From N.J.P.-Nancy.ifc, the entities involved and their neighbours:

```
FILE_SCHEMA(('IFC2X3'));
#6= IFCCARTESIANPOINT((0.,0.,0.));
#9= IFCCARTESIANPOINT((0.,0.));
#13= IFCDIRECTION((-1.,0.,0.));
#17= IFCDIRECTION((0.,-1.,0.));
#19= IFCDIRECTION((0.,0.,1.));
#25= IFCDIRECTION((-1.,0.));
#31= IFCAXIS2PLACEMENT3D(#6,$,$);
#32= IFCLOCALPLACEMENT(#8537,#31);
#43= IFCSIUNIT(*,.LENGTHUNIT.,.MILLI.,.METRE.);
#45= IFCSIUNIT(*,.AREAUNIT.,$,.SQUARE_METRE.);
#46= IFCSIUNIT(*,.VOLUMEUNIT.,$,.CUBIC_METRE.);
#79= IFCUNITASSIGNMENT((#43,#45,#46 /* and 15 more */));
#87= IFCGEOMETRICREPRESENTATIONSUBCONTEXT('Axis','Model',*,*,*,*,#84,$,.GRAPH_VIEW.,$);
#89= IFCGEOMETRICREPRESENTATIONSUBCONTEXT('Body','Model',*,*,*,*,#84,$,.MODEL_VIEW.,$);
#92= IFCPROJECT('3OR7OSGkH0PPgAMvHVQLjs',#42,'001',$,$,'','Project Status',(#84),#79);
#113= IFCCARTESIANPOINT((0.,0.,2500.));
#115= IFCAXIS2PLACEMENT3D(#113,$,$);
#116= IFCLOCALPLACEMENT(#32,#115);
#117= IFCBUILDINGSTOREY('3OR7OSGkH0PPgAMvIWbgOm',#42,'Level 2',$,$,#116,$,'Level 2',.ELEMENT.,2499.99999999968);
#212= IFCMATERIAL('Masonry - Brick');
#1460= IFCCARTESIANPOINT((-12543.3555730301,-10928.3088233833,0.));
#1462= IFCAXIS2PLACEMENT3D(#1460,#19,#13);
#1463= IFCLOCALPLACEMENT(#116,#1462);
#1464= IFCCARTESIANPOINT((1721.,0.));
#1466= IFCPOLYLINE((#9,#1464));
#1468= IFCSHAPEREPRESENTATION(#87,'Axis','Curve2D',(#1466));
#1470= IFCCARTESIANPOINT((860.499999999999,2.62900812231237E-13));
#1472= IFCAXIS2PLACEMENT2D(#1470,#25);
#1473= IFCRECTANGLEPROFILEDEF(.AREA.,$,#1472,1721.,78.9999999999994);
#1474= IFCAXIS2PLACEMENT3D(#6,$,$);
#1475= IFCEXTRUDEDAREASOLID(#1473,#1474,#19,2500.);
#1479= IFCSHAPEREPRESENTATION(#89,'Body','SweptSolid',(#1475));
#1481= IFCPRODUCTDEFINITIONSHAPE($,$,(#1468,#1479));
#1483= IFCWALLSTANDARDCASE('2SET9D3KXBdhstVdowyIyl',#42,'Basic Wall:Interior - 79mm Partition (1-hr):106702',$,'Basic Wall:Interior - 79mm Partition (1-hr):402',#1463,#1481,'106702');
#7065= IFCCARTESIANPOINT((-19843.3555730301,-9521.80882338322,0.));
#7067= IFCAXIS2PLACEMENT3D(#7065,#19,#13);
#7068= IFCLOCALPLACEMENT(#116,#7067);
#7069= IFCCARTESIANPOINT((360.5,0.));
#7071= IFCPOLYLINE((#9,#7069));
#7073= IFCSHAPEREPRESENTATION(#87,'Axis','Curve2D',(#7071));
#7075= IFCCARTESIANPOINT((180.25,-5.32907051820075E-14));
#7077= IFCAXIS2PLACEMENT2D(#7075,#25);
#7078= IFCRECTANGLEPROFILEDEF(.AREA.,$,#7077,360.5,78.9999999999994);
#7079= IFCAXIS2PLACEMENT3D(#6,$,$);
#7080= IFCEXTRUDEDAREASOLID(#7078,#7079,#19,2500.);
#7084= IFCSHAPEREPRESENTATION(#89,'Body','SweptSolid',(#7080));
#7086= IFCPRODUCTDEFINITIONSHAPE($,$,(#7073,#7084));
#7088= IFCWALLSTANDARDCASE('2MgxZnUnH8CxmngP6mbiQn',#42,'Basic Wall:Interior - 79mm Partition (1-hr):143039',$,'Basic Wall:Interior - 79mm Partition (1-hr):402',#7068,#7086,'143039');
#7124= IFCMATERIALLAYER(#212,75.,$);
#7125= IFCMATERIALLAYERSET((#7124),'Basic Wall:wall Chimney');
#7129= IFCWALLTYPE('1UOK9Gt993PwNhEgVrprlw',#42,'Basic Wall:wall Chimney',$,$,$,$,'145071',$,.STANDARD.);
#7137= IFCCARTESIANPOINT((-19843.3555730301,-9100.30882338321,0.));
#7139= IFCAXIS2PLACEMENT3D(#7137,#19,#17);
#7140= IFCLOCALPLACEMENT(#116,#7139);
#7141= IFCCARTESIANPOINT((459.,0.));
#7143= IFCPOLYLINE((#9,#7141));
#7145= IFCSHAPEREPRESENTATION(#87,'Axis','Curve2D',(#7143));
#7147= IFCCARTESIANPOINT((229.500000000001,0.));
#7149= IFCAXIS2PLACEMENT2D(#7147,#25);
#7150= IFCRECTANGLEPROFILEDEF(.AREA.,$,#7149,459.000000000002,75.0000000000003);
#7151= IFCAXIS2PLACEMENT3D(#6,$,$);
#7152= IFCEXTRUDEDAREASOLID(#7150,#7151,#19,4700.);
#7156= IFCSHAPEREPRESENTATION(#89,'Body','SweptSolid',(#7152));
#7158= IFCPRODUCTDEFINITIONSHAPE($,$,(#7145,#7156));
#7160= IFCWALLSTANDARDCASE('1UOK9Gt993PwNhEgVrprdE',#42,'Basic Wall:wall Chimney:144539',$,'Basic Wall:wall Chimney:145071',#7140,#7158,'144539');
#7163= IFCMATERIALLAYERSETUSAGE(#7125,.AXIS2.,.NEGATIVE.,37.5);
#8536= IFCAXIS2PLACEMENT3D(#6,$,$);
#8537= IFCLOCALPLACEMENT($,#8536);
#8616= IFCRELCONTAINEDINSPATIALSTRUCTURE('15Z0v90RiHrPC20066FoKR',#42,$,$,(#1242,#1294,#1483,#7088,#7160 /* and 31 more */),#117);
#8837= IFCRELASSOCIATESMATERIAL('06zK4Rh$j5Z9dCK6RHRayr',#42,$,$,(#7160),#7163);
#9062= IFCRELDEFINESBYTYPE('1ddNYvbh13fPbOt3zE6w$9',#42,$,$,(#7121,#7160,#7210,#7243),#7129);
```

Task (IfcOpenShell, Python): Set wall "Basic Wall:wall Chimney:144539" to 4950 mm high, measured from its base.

```python
import ifcopenshell
import ifcopenshell.geom
import ifcopenshell.util.representation
import ifcopenshell.util.shape
import ifcopenshell.util.unit

model = ifcopenshell.open("N.J.P.-Nancy.ifc")
unit_scale = ifcopenshell.util.unit.calculate_unit_scale(model)
settings = ifcopenshell.geom.settings()


def volume(element):
    """Net volume in cubic metres, openings subtracted."""
    shape = ifcopenshell.geom.create_shape(settings, element)
    return ifcopenshell.util.shape.get_volume(shape.geometry)


wall = model.by_id(7160)
before = volume(wall)

body = ifcopenshell.util.representation.get_representation(wall, "Model", "Body")
solid = body.Items[0]
old_height = solid.Depth
solid.Depth = 4.95 / unit_scale
after = volume(wall)

print(f"height {old_height:g} -> {solid.Depth:g}, volume {before:.3f} -> {after:.3f} m3")

model.write("N.J.P.-Nancy_v2.ifc")
```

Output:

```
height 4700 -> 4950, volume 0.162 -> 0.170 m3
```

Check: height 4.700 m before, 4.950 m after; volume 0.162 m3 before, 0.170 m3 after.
